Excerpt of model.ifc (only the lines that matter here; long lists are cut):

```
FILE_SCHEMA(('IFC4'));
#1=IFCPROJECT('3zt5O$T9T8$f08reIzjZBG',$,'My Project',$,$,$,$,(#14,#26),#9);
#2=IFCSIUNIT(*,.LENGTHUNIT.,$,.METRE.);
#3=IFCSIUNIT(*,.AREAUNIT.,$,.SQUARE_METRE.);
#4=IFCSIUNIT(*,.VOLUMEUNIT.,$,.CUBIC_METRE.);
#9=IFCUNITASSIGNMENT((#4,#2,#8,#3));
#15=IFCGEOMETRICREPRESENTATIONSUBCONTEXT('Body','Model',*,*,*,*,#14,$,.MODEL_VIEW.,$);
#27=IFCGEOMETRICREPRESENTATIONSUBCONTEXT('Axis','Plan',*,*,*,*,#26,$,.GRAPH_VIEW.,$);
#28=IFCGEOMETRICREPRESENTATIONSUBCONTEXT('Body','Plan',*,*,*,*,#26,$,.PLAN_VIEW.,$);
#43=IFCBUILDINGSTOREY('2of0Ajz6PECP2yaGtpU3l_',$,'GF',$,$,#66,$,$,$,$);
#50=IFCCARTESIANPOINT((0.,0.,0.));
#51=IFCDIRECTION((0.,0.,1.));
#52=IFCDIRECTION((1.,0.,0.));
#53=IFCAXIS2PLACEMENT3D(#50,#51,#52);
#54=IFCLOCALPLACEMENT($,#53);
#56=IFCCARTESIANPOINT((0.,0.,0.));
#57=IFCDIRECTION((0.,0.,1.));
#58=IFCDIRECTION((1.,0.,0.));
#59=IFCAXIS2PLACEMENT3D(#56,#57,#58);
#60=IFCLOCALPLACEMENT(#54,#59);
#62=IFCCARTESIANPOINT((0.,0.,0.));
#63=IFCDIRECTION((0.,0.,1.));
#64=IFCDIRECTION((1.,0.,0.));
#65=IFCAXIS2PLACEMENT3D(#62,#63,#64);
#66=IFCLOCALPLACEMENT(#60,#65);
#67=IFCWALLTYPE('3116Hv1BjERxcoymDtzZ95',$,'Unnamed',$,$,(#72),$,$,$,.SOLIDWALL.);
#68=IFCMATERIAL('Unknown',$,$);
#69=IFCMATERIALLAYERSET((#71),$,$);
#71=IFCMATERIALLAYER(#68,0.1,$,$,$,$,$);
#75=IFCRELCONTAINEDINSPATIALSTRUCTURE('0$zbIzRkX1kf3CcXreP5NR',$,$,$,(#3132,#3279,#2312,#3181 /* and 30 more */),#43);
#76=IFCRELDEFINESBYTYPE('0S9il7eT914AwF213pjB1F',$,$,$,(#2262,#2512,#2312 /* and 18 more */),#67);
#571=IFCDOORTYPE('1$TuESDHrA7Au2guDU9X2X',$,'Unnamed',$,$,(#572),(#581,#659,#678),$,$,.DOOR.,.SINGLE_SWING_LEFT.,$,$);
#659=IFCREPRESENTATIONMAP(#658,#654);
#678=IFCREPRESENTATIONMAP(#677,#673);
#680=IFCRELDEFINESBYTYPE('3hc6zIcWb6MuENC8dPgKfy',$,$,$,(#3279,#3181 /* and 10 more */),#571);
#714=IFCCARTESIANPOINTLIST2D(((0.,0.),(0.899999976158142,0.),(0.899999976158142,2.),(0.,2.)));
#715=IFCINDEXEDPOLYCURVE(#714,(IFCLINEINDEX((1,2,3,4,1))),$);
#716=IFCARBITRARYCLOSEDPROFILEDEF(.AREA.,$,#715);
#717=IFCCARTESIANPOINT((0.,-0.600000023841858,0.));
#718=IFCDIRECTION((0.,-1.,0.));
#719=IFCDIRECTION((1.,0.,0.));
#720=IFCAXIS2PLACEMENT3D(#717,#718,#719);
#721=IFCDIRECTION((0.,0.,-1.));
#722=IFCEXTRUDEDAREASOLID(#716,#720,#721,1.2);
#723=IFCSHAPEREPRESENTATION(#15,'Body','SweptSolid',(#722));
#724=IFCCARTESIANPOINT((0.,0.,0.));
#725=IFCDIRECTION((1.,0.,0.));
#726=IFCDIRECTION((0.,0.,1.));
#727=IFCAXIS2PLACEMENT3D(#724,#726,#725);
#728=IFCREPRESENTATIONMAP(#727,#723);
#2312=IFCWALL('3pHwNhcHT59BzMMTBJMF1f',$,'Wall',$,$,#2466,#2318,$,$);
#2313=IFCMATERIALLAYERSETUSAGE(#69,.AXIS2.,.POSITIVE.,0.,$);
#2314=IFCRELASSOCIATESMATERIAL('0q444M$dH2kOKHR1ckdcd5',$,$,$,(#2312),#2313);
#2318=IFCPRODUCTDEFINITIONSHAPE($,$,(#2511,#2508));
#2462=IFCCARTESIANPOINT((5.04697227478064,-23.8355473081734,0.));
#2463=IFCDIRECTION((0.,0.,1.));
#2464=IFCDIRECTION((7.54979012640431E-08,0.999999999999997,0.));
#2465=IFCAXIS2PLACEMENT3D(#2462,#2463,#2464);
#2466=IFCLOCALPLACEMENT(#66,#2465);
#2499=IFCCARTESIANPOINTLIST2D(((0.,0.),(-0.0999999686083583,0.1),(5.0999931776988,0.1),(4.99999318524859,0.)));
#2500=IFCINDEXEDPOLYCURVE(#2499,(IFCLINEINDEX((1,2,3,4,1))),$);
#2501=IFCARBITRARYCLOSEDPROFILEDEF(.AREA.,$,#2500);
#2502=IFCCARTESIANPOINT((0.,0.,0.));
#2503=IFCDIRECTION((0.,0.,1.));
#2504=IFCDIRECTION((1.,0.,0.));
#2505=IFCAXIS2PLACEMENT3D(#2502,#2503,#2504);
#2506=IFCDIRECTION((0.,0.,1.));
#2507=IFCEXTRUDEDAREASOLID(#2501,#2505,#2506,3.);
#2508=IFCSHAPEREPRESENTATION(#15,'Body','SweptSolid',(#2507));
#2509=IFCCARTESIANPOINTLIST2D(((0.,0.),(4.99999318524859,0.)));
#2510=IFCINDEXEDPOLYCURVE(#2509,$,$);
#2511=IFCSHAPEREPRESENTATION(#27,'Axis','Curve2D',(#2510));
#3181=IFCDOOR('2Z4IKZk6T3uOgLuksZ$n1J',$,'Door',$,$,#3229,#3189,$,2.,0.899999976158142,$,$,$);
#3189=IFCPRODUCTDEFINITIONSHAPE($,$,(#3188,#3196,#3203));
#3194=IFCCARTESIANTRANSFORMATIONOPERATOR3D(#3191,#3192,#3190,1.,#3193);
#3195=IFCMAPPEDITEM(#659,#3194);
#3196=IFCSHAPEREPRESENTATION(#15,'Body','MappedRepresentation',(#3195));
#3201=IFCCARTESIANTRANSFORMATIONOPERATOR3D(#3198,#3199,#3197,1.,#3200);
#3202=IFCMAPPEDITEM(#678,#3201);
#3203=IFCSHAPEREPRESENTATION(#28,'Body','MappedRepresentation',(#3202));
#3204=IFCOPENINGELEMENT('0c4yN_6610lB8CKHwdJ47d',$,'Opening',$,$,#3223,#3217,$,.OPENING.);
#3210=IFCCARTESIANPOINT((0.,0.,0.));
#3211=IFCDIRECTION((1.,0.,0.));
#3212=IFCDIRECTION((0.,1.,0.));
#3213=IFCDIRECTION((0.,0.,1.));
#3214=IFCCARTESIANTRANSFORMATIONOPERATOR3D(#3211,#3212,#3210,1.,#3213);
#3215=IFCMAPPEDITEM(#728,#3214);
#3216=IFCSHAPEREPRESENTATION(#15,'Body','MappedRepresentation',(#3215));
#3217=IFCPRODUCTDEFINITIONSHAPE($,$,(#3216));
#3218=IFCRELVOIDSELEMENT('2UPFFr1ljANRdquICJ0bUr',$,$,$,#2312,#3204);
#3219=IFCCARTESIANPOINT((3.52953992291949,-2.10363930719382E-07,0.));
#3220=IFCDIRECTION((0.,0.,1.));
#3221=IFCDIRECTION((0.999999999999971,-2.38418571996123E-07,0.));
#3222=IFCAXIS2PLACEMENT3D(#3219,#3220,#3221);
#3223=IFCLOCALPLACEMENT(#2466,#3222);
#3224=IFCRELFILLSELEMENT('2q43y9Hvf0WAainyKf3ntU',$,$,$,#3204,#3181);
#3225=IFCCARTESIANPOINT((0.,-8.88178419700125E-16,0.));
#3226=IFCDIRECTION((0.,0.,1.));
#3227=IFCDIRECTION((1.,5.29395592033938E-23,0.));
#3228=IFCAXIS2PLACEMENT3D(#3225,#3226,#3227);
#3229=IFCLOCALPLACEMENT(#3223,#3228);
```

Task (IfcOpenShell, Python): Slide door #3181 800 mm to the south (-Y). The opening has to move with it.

```python
import ifcopenshell
import ifcopenshell.api.geometry
import ifcopenshell.util.placement
import ifcopenshell.util.unit

model = ifcopenshell.open("model.ifc")
unit_scale = ifcopenshell.util.unit.calculate_unit_scale(model)

door = model.by_guid("2Z4IKZk6T3uOgLuksZ$n1J")
opening = door.FillsVoids[0].RelatingOpeningElement
wall = opening.VoidsElements[0].RelatingBuildingElement

wall_matrix = ifcopenshell.util.placement.get_local_placement(wall.ObjectPlacement)
shift = wall_matrix[:3, 0] * -0.8 / unit_scale
before = ifcopenshell.util.placement.get_local_placement(door.ObjectPlacement)[:3, 3].copy()

# The door is placed relative to its opening, so it follows when the opening moves.
matrix = ifcopenshell.util.placement.get_local_placement(opening.ObjectPlacement)
matrix[:3, 3] += shift
ifcopenshell.api.geometry.edit_object_placement(
    model, product=opening, matrix=matrix, is_si=False, should_transform_children=True
)

after = ifcopenshell.util.placement.get_local_placement(door.ObjectPlacement)[:3, 3]
print("door moved by", (after - before).round(3) + 0.0)

model.write("model_updated.ifc")
```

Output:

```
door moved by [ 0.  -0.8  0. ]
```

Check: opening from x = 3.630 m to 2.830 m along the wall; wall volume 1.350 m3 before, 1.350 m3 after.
